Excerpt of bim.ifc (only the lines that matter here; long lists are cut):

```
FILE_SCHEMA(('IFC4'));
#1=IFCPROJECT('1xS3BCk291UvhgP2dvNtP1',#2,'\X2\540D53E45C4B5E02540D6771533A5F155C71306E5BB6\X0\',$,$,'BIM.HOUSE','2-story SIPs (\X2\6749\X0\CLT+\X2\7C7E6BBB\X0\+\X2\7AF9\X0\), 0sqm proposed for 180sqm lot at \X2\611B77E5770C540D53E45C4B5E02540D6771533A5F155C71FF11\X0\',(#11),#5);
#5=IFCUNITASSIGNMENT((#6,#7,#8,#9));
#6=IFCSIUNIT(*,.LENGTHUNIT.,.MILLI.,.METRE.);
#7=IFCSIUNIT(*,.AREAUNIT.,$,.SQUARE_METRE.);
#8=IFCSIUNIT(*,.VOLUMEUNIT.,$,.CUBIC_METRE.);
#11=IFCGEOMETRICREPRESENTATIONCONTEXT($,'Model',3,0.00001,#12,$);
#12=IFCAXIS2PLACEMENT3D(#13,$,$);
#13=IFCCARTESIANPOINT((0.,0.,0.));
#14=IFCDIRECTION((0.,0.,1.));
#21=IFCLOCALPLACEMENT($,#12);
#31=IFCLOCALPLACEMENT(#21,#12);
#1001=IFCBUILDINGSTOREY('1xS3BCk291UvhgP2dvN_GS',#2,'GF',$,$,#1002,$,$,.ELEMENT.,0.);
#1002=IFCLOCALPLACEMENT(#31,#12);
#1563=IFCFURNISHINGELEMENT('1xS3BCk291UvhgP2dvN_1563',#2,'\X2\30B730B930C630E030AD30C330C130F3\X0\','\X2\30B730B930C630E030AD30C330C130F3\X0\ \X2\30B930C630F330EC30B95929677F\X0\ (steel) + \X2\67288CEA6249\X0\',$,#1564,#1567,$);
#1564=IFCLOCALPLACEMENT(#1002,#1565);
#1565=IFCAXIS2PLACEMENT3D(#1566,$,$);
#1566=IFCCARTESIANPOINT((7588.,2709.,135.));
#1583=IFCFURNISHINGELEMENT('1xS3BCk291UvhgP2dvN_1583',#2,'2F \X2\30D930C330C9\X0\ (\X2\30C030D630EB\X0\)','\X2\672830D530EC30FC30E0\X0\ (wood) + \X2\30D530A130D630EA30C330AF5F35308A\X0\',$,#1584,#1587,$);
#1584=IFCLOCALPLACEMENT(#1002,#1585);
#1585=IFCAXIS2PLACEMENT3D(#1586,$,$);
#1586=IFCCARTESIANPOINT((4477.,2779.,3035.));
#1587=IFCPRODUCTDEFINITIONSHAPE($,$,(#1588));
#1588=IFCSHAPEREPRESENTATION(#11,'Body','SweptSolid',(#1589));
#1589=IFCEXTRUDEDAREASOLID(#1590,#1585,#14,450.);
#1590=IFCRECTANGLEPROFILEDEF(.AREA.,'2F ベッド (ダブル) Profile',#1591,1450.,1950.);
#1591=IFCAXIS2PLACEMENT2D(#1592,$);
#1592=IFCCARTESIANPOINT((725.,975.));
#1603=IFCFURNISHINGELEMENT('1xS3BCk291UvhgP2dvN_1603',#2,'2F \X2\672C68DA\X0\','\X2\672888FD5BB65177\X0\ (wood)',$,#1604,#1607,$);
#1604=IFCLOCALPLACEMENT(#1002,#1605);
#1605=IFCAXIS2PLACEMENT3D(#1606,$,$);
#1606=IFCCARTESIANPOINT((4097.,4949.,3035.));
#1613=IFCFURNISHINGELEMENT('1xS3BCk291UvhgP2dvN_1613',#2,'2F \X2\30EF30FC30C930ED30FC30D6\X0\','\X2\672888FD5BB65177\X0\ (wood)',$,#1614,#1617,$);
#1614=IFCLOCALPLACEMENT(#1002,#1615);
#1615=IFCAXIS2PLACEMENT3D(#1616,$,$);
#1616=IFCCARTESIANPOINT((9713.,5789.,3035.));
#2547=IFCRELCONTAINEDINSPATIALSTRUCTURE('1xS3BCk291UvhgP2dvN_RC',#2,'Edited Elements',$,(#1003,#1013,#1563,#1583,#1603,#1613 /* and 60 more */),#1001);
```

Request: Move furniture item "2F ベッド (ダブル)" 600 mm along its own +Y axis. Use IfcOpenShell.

```python
import ifcopenshell
import ifcopenshell.api.geometry
import ifcopenshell.util.placement

model = ifcopenshell.open("bim.ifc")

item = model.by_id(1583)
matrix = ifcopenshell.util.placement.get_local_placement(item.ObjectPlacement)
matrix[:3, 3] += matrix[:3, 1] * 600.0
ifcopenshell.api.geometry.edit_object_placement(model, product=item, matrix=matrix, is_si=False)

print(ifcopenshell.util.placement.get_local_placement(item.ObjectPlacement).round(3) + 0.0)

model.write("bim_edited.ifc")
```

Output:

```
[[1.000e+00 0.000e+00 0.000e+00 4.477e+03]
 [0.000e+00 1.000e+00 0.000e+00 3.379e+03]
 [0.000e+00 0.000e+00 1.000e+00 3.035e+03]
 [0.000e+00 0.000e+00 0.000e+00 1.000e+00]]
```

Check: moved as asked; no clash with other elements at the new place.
